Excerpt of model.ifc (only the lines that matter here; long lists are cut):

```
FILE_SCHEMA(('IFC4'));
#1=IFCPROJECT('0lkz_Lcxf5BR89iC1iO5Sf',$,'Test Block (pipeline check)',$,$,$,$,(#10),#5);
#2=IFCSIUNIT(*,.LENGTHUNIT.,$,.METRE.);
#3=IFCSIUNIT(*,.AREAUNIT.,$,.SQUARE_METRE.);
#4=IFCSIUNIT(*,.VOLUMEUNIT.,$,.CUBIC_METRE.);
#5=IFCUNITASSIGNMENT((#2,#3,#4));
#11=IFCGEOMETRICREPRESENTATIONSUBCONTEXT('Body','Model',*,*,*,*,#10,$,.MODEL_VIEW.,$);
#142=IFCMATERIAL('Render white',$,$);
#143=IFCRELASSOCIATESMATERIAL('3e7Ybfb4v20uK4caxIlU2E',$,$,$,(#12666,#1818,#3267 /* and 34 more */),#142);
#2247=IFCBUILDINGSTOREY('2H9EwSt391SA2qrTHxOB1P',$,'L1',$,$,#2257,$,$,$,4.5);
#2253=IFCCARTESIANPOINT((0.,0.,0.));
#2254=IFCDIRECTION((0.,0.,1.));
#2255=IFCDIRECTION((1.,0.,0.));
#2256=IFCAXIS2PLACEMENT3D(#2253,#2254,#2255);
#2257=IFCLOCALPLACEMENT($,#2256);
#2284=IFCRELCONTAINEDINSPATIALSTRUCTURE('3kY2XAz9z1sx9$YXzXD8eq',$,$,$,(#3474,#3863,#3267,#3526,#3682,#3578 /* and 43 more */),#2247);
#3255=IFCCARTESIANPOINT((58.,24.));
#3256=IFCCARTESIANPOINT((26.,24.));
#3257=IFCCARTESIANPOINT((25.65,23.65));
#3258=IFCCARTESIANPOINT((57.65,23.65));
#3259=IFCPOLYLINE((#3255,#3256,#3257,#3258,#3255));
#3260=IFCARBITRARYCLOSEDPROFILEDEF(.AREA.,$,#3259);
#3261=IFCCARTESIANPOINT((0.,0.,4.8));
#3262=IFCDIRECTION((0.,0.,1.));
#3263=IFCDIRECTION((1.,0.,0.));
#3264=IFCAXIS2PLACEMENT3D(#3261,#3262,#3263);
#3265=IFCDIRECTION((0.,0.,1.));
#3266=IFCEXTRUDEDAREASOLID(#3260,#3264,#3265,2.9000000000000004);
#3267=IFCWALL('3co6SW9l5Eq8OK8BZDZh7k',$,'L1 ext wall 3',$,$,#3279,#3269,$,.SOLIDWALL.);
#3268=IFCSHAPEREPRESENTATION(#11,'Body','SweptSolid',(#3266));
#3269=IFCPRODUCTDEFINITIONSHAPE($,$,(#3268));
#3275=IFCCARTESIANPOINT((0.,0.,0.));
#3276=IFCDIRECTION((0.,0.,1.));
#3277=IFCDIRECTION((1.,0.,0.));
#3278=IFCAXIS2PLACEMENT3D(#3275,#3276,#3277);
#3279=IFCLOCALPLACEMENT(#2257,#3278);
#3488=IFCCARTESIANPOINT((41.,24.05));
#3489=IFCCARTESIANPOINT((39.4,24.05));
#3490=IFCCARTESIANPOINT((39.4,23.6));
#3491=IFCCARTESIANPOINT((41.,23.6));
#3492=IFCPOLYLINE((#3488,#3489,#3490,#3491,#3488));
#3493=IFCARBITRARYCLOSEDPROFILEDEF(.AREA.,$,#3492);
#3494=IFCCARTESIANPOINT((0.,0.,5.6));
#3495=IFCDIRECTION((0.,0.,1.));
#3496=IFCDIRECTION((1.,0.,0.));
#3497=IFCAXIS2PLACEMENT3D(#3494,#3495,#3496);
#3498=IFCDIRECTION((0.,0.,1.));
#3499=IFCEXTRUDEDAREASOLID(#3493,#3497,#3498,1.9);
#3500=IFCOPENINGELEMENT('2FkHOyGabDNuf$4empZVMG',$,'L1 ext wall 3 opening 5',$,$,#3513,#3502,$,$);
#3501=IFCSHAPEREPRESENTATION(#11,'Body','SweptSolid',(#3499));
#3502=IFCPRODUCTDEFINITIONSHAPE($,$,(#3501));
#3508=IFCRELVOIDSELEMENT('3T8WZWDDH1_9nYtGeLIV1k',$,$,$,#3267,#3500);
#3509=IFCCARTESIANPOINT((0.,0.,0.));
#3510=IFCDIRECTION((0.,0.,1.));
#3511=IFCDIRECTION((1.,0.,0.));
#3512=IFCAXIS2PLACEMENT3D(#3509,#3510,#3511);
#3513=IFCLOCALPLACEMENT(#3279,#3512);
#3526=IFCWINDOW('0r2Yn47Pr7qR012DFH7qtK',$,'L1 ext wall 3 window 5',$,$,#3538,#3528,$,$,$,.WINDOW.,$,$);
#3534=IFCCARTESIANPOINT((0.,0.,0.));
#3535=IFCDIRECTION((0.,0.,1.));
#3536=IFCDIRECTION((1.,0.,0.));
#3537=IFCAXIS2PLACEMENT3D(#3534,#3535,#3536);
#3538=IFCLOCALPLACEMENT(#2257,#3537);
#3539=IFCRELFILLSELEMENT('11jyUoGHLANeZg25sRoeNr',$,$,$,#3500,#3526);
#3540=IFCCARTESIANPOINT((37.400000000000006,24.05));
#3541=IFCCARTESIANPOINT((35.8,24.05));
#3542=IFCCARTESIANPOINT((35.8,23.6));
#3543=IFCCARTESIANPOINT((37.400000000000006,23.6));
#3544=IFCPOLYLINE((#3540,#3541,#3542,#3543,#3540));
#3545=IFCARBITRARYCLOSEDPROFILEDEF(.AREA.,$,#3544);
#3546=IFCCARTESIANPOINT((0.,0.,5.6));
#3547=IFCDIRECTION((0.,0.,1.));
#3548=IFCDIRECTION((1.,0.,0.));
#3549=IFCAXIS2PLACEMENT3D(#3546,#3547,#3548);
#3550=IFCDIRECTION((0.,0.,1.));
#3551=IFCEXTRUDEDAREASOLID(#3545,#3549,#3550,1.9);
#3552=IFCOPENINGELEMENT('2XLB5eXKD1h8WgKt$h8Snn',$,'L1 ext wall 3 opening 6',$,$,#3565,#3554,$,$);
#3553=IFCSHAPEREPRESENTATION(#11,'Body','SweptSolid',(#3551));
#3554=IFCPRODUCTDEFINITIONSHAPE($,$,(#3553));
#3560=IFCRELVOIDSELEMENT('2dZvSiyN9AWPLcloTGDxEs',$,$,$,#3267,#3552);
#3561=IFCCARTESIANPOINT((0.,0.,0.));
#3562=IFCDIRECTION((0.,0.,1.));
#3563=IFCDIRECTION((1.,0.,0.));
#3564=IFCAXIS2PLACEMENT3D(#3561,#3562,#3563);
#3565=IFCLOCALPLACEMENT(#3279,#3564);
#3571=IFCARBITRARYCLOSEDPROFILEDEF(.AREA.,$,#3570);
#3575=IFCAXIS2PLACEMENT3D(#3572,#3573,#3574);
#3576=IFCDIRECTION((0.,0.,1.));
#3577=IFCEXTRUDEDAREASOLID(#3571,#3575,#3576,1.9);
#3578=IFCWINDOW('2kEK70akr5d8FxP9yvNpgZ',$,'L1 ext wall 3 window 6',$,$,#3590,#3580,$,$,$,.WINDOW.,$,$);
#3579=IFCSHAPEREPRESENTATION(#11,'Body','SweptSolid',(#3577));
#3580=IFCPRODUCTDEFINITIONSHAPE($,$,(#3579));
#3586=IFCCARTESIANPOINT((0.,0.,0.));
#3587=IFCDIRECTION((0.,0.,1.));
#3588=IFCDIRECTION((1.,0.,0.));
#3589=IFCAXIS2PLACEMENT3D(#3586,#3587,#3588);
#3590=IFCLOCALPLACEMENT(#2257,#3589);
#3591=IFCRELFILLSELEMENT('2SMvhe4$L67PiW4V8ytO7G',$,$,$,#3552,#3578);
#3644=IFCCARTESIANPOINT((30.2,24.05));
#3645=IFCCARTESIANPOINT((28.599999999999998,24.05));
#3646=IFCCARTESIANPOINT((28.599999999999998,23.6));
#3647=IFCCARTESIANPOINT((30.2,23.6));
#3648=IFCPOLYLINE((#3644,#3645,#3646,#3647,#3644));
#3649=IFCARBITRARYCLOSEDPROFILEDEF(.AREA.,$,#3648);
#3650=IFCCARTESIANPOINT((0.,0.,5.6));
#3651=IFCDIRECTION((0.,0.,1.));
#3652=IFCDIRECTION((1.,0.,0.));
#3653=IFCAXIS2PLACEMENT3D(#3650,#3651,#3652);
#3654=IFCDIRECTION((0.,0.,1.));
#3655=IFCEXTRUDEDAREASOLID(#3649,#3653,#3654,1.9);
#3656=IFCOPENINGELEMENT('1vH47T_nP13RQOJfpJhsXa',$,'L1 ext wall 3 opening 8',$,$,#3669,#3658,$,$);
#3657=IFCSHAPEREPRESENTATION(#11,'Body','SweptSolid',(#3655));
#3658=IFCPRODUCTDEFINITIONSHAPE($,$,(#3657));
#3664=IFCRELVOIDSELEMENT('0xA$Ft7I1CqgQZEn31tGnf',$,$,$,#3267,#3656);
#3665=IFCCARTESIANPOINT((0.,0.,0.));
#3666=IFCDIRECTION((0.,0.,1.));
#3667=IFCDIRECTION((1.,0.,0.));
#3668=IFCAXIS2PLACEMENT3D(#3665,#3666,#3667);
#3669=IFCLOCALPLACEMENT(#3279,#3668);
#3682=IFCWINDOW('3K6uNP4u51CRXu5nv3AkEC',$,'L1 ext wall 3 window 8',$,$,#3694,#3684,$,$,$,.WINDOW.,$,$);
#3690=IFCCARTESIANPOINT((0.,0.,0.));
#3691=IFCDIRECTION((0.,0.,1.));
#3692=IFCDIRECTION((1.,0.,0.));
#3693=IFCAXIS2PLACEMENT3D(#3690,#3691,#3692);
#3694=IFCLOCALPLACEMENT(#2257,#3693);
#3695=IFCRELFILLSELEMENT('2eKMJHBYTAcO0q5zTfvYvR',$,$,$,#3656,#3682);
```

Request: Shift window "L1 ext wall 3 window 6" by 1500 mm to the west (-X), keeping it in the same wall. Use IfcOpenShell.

```python
import ifcopenshell
import ifcopenshell.api.geometry
import ifcopenshell.util.placement
import ifcopenshell.util.unit

model = ifcopenshell.open("model.ifc")
unit_scale = ifcopenshell.util.unit.calculate_unit_scale(model)

window = model.by_guid("2kEK70akr5d8FxP9yvNpgZ")
opening = window.FillsVoids[0].RelatingOpeningElement
wall = opening.VoidsElements[0].RelatingBuildingElement

wall_matrix = ifcopenshell.util.placement.get_local_placement(wall.ObjectPlacement)
shift = wall_matrix[:3, 0] * -1.5 / unit_scale
before = ifcopenshell.util.placement.get_local_placement(window.ObjectPlacement)[:3, 3].copy()

# The window is not placed relative to its opening, so move both.
for product in (opening, window):
    matrix = ifcopenshell.util.placement.get_local_placement(product.ObjectPlacement)
    matrix[:3, 3] += shift
    ifcopenshell.api.geometry.edit_object_placement(model, product=product, matrix=matrix, is_si=False)

after = ifcopenshell.util.placement.get_local_placement(window.ObjectPlacement)[:3, 3]
print("window moved by", (after - before).round(3) + 0.0)

model.write("model-out.ifc")
```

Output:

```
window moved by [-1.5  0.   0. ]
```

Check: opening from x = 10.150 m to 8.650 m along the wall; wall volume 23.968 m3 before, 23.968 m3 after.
